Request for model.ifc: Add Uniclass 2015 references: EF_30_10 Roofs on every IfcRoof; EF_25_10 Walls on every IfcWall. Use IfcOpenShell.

First a look at what the model holds.

```python
import ifcopenshell

model = ifcopenshell.open("model.ifc")
print(model.schema)
print("classifications:", [c.Name for c in model.by_type("IfcClassification")])
for ifc_class in ("IfcDoor", "IfcRoof", "IfcStair", "IfcWall", "IfcWindow"):
    print(ifc_class, len(model.by_type(ifc_class)))
```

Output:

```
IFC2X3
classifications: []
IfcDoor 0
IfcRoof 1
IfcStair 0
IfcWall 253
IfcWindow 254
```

```python
import ifcopenshell
import ifcopenshell.api.classification

model = ifcopenshell.open("model.ifc")

# IFC2X3 requires Source and Edition and has no link from the project to the system.
system = model.create_entity("IfcClassification", Source="NBS", Edition="2015", Name="Uniclass 2015")

codes = {
    "IfcRoof": ("EF_30_10", "Roofs"),
    "IfcWall": ("EF_25_10", "Walls"),
}
for ifc_class, (code, name) in codes.items():
    products = model.by_type(ifc_class)
    ifcopenshell.api.classification.add_reference(
        model, products=products, classification=system, identification=code, name=name
    )
    print(code, len(products))

model.write("model_rev.ifc")
```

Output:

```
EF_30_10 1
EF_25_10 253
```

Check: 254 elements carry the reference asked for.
